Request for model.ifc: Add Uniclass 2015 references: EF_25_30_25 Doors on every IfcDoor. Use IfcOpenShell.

First a look at what the model holds.

```python
import ifcopenshell

model = ifcopenshell.open("model.ifc")
print(model.schema)
print("classifications:", [c.Name for c in model.by_type("IfcClassification")])
for ifc_class in ("IfcDoor", "IfcRoof", "IfcStair", "IfcWall", "IfcWindow"):
    print(ifc_class, len(model.by_type(ifc_class)))
```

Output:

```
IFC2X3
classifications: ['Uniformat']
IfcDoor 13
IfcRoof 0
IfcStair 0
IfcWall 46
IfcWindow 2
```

```python
import ifcopenshell
import ifcopenshell.api.classification

model = ifcopenshell.open("model.ifc")

# IFC2X3 requires Source and Edition and has no link from the project to the system.
system = model.create_entity("IfcClassification", Source="NBS", Edition="2015", Name="Uniclass 2015")

codes = {
    "IfcDoor": ("EF_25_30_25", "Doors"),
}
for ifc_class, (code, name) in codes.items():
    products = model.by_type(ifc_class)
    ifcopenshell.api.classification.add_reference(
        model, products=products, classification=system, identification=code, name=name
    )
    print(code, len(products))

model.write("model-out.ifc")
```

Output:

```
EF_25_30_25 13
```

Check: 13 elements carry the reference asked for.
